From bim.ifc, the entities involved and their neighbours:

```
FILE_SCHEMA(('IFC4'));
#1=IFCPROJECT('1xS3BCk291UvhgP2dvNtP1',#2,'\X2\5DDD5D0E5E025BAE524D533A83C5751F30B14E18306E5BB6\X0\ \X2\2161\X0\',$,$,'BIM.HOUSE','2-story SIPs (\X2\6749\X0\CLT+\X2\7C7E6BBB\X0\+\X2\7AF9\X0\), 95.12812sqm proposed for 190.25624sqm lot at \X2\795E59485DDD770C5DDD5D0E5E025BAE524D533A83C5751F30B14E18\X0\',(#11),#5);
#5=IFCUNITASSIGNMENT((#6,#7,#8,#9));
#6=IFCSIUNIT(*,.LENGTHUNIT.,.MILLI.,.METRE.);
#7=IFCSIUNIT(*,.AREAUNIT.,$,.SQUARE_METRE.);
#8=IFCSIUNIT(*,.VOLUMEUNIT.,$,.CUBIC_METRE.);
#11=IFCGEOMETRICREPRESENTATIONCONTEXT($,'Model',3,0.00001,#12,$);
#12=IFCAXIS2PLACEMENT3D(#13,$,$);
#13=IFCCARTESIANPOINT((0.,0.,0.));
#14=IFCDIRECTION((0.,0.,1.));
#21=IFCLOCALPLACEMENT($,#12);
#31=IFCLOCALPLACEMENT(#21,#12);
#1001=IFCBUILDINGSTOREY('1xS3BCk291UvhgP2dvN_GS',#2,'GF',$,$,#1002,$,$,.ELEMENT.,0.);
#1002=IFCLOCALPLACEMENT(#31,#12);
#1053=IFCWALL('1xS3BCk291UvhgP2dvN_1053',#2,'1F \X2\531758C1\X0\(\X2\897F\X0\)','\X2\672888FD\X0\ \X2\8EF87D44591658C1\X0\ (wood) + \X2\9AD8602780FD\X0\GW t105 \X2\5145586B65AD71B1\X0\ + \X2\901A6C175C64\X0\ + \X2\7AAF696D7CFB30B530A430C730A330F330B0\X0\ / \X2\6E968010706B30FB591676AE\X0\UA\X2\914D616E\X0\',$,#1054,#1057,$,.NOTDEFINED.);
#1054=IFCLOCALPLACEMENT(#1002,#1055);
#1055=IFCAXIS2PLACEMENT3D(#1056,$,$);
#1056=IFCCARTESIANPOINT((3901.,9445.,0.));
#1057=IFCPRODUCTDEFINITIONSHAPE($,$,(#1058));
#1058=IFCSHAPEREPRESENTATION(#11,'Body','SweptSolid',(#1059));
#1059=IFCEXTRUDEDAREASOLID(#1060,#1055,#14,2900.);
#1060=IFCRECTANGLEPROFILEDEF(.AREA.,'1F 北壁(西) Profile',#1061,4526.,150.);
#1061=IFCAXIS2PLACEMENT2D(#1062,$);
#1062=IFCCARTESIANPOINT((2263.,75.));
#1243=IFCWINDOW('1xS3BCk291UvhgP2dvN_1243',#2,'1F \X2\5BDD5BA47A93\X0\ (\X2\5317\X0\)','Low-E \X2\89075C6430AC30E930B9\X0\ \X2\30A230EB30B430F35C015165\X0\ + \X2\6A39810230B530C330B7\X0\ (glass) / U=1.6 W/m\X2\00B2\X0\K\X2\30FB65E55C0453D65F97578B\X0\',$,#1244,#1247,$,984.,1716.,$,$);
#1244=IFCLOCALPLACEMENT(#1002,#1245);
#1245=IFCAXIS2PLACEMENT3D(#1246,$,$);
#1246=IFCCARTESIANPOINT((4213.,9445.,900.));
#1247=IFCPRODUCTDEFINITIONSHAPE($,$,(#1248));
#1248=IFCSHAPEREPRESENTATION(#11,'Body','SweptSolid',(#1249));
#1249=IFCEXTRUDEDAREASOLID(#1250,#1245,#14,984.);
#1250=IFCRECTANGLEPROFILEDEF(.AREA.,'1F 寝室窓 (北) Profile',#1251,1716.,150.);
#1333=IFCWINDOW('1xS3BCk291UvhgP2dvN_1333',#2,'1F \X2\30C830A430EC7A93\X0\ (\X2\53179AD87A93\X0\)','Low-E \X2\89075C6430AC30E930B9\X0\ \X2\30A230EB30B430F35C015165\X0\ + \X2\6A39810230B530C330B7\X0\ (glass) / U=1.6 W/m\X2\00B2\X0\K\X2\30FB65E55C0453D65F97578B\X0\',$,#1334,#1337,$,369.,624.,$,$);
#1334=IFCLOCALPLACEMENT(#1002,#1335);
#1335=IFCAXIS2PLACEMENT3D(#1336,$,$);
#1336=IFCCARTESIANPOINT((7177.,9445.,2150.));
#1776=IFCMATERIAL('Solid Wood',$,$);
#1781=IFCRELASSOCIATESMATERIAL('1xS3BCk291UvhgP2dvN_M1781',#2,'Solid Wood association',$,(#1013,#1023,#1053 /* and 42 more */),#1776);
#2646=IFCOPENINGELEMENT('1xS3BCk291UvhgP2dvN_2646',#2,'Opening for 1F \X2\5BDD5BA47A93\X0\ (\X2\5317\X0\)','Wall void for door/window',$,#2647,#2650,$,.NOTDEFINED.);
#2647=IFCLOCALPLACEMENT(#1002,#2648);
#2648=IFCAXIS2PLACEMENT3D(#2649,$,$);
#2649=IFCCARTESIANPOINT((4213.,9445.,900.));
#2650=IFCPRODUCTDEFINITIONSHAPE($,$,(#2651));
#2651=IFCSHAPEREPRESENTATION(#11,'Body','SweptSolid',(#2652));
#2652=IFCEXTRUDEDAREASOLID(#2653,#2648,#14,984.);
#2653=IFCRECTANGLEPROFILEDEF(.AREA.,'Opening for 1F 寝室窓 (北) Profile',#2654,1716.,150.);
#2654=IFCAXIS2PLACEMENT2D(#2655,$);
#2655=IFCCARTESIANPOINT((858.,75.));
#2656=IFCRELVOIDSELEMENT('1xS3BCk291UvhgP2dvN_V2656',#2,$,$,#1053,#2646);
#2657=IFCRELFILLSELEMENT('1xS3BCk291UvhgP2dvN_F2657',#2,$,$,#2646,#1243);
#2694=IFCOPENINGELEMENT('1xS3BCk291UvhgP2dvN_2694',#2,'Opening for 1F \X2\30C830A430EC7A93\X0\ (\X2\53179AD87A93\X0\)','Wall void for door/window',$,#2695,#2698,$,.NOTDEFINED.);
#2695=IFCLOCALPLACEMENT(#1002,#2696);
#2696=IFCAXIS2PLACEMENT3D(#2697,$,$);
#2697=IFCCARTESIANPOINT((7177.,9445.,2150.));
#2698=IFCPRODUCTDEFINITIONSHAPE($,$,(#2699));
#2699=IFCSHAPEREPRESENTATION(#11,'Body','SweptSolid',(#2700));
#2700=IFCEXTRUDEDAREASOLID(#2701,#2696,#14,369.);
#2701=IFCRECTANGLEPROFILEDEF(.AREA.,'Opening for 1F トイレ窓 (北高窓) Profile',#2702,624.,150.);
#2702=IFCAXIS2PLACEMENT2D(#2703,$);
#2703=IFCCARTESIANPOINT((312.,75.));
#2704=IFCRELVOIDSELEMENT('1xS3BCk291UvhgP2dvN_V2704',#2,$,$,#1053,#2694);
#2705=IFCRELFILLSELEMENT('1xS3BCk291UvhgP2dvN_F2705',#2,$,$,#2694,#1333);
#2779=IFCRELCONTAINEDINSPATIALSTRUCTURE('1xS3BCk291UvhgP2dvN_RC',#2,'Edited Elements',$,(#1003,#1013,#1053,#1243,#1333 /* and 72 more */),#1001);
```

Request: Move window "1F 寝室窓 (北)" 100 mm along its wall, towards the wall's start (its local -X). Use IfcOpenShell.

```python
import ifcopenshell
import ifcopenshell.api.geometry
import ifcopenshell.util.placement
import ifcopenshell.util.unit

model = ifcopenshell.open("bim.ifc")
unit_scale = ifcopenshell.util.unit.calculate_unit_scale(model)

window = model.by_guid("1xS3BCk291UvhgP2dvN_1243")
opening = window.FillsVoids[0].RelatingOpeningElement
wall = opening.VoidsElements[0].RelatingBuildingElement

wall_matrix = ifcopenshell.util.placement.get_local_placement(wall.ObjectPlacement)
shift = wall_matrix[:3, 0] * -0.1 / unit_scale
before = ifcopenshell.util.placement.get_local_placement(window.ObjectPlacement)[:3, 3].copy()

# The window is not placed relative to its opening, so move both.
for product in (opening, window):
    matrix = ifcopenshell.util.placement.get_local_placement(product.ObjectPlacement)
    matrix[:3, 3] += shift
    ifcopenshell.api.geometry.edit_object_placement(model, product=product, matrix=matrix, is_si=False)

after = ifcopenshell.util.placement.get_local_placement(window.ObjectPlacement)[:3, 3]
print("window moved by", (after - before).round(3) + 0.0)

model.write("bim_rev.ifc")
```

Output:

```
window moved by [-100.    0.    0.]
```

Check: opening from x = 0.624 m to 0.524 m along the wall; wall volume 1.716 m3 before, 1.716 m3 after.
